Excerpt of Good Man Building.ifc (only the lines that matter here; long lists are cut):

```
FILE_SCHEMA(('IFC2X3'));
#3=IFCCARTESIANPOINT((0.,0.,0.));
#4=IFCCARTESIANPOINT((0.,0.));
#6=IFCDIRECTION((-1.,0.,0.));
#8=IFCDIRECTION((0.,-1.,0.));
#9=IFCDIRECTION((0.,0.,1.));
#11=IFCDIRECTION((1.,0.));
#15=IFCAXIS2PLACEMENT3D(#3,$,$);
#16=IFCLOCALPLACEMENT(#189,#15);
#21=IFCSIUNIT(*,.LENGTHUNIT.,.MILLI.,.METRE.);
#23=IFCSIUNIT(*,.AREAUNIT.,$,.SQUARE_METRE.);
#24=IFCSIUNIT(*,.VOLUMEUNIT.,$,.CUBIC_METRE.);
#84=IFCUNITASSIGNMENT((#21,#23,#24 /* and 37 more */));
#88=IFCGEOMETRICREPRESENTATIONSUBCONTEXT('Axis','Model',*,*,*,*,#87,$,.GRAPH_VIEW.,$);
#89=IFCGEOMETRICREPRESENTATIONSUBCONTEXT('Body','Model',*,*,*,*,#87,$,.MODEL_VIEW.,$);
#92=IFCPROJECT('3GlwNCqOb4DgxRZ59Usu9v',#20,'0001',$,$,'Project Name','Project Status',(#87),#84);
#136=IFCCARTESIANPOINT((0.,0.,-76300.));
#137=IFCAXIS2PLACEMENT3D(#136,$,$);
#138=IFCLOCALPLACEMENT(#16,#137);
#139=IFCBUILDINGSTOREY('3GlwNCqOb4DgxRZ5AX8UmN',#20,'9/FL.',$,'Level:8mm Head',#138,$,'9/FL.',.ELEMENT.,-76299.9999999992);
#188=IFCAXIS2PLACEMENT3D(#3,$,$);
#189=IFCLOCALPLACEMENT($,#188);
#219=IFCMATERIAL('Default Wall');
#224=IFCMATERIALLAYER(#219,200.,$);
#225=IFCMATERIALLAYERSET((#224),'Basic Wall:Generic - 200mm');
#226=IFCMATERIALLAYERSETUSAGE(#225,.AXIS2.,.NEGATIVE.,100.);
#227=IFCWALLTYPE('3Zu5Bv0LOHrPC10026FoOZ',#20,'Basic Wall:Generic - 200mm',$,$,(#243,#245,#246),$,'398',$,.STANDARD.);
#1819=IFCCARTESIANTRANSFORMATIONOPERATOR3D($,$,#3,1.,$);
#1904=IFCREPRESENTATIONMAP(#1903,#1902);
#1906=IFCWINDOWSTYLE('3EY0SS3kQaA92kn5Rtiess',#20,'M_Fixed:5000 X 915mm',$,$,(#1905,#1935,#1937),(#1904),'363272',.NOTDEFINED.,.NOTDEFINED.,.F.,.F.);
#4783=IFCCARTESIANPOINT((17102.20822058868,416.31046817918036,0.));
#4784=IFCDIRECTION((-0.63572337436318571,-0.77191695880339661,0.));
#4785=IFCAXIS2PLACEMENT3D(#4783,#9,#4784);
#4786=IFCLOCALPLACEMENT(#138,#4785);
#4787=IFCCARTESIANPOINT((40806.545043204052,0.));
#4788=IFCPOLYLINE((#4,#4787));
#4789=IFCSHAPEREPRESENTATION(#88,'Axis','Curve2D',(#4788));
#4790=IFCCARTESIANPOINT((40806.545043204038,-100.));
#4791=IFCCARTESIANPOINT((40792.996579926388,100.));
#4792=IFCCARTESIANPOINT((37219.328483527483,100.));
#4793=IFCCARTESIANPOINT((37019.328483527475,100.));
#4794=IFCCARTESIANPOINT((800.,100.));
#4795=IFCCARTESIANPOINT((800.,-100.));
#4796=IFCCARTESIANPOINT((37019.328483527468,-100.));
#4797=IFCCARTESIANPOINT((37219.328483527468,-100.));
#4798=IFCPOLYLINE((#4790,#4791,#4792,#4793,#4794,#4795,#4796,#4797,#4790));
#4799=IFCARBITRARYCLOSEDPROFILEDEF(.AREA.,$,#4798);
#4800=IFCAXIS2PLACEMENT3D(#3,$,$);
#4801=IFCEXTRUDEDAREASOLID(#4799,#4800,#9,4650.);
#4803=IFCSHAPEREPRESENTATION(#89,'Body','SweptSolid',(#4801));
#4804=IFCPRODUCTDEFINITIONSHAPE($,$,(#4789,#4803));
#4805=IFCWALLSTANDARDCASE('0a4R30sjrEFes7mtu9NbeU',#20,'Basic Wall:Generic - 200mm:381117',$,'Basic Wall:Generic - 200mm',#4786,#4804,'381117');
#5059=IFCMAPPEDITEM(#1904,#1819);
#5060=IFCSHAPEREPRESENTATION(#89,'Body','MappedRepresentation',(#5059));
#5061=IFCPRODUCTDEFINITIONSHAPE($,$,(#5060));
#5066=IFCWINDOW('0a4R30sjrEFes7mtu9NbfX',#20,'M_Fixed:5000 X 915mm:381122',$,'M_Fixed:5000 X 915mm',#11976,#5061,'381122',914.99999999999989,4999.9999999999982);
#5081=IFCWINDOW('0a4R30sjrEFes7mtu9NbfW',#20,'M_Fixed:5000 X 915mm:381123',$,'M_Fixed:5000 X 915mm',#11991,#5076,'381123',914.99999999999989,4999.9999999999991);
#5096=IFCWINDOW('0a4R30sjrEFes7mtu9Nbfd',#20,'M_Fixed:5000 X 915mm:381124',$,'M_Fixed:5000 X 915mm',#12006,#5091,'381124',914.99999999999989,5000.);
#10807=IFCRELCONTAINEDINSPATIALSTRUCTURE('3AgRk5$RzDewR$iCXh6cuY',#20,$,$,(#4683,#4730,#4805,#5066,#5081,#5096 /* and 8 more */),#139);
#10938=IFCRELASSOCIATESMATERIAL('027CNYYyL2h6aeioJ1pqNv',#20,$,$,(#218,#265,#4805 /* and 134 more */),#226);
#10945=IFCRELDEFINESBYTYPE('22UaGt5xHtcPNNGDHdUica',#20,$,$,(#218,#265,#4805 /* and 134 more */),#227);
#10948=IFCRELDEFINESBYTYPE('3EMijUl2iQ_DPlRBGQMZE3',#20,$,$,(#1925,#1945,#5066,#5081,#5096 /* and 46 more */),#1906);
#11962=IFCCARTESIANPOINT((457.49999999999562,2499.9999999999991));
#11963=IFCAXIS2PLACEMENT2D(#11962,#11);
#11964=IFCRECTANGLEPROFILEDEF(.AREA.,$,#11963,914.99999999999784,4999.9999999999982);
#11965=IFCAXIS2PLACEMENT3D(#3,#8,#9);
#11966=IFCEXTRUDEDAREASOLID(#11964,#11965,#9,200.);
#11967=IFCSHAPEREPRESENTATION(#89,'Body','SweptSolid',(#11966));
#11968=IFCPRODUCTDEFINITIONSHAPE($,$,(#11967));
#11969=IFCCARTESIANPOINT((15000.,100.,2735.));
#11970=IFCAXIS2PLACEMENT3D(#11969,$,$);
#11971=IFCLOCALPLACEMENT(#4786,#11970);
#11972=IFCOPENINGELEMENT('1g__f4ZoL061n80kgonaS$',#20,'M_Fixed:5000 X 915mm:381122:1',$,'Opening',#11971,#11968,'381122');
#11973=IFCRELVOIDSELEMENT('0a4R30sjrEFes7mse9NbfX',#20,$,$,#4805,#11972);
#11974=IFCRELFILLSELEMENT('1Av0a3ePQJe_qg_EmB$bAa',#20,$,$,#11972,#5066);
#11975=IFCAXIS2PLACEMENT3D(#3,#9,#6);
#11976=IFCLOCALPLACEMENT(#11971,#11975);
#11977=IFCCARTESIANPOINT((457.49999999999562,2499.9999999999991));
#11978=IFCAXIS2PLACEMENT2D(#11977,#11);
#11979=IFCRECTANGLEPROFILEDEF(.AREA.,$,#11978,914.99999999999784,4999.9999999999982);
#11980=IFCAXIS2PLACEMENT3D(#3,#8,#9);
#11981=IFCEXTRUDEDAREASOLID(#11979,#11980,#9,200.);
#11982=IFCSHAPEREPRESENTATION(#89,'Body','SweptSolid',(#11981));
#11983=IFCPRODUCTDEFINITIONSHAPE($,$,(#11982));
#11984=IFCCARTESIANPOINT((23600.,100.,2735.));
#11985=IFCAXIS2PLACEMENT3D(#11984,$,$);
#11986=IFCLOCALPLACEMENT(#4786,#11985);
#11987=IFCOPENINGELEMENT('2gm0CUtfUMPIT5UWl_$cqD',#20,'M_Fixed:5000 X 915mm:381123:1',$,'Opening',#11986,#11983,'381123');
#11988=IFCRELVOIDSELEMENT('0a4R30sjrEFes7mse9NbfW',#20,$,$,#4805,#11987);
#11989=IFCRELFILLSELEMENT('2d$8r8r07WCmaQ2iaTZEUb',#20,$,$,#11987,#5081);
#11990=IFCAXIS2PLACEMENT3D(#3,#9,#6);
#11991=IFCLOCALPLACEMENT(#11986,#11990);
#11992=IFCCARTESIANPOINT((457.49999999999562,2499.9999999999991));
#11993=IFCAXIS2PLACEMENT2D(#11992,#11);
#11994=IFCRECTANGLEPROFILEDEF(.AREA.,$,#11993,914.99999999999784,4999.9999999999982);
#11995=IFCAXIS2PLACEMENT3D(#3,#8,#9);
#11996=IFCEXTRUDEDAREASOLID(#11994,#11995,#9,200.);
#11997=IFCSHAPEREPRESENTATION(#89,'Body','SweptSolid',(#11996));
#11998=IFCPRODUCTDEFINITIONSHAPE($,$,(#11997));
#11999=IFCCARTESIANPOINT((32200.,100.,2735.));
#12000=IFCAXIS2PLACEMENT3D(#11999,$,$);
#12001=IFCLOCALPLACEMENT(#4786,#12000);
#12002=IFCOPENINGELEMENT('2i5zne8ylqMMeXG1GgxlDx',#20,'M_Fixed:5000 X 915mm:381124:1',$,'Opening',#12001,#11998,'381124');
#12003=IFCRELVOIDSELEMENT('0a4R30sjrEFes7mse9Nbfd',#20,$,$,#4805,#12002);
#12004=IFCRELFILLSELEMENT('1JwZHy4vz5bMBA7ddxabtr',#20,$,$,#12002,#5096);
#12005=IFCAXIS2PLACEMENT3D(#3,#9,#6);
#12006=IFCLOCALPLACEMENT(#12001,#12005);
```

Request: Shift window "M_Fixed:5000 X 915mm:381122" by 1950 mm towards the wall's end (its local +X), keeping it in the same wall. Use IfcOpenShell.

```python
import ifcopenshell
import ifcopenshell.api.geometry
import ifcopenshell.util.placement
import ifcopenshell.util.unit

model = ifcopenshell.open("Good Man Building.ifc")
unit_scale = ifcopenshell.util.unit.calculate_unit_scale(model)

window = model.by_guid("0a4R30sjrEFes7mtu9NbfX")
opening = window.FillsVoids[0].RelatingOpeningElement
wall = opening.VoidsElements[0].RelatingBuildingElement

wall_matrix = ifcopenshell.util.placement.get_local_placement(wall.ObjectPlacement)
shift = wall_matrix[:3, 0] * 1.95 / unit_scale
before = ifcopenshell.util.placement.get_local_placement(window.ObjectPlacement)[:3, 3].copy()

# The window is placed relative to its opening, so it follows when the opening moves.
matrix = ifcopenshell.util.placement.get_local_placement(opening.ObjectPlacement)
matrix[:3, 3] += shift
ifcopenshell.api.geometry.edit_object_placement(
    model, product=opening, matrix=matrix, is_si=False, should_transform_children=True
)

after = ifcopenshell.util.placement.get_local_placement(window.ObjectPlacement)[:3, 3]
print("window moved by", (after - before).round(3) + 0.0)

model.write("Good Man Building_updated.ifc")
```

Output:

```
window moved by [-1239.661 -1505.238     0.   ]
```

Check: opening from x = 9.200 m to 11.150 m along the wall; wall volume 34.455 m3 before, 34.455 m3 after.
